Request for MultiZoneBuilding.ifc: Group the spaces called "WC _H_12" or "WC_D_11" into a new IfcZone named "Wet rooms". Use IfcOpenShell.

First a look at what the model holds.

```python
import ifcopenshell

model = ifcopenshell.open("MultiZoneBuilding.ifc")
print(model.schema)
seen = {}
for space in model.by_type("IfcSpace"):
    seen[space.LongName] = seen.get(space.LongName, 0) + 1
for name, count in sorted(seen.items(), key=str):
    print(count, "x", name)
print("zones:", [z.Name for z in model.by_type("IfcZone")][:20])
```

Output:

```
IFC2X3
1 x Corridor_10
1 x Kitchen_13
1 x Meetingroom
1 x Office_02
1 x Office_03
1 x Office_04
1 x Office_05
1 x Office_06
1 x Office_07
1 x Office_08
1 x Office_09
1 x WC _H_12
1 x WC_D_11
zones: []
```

```python
import ifcopenshell
import ifcopenshell.api.group
import ifcopenshell.api.root

model = ifcopenshell.open("MultiZoneBuilding.ifc")

names = {"WC _H_12", "WC_D_11"}
spaces = [s for s in model.by_type("IfcSpace") if s.LongName in names]

zone = ifcopenshell.api.root.create_entity(model, ifc_class="IfcZone", name="Wet rooms")
ifcopenshell.api.group.assign_group(model, products=spaces, group=zone)
print(len(spaces), "spaces in", zone.Name)

model.write("MultiZoneBuilding-out.ifc")
```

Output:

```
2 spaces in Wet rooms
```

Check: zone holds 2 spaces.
